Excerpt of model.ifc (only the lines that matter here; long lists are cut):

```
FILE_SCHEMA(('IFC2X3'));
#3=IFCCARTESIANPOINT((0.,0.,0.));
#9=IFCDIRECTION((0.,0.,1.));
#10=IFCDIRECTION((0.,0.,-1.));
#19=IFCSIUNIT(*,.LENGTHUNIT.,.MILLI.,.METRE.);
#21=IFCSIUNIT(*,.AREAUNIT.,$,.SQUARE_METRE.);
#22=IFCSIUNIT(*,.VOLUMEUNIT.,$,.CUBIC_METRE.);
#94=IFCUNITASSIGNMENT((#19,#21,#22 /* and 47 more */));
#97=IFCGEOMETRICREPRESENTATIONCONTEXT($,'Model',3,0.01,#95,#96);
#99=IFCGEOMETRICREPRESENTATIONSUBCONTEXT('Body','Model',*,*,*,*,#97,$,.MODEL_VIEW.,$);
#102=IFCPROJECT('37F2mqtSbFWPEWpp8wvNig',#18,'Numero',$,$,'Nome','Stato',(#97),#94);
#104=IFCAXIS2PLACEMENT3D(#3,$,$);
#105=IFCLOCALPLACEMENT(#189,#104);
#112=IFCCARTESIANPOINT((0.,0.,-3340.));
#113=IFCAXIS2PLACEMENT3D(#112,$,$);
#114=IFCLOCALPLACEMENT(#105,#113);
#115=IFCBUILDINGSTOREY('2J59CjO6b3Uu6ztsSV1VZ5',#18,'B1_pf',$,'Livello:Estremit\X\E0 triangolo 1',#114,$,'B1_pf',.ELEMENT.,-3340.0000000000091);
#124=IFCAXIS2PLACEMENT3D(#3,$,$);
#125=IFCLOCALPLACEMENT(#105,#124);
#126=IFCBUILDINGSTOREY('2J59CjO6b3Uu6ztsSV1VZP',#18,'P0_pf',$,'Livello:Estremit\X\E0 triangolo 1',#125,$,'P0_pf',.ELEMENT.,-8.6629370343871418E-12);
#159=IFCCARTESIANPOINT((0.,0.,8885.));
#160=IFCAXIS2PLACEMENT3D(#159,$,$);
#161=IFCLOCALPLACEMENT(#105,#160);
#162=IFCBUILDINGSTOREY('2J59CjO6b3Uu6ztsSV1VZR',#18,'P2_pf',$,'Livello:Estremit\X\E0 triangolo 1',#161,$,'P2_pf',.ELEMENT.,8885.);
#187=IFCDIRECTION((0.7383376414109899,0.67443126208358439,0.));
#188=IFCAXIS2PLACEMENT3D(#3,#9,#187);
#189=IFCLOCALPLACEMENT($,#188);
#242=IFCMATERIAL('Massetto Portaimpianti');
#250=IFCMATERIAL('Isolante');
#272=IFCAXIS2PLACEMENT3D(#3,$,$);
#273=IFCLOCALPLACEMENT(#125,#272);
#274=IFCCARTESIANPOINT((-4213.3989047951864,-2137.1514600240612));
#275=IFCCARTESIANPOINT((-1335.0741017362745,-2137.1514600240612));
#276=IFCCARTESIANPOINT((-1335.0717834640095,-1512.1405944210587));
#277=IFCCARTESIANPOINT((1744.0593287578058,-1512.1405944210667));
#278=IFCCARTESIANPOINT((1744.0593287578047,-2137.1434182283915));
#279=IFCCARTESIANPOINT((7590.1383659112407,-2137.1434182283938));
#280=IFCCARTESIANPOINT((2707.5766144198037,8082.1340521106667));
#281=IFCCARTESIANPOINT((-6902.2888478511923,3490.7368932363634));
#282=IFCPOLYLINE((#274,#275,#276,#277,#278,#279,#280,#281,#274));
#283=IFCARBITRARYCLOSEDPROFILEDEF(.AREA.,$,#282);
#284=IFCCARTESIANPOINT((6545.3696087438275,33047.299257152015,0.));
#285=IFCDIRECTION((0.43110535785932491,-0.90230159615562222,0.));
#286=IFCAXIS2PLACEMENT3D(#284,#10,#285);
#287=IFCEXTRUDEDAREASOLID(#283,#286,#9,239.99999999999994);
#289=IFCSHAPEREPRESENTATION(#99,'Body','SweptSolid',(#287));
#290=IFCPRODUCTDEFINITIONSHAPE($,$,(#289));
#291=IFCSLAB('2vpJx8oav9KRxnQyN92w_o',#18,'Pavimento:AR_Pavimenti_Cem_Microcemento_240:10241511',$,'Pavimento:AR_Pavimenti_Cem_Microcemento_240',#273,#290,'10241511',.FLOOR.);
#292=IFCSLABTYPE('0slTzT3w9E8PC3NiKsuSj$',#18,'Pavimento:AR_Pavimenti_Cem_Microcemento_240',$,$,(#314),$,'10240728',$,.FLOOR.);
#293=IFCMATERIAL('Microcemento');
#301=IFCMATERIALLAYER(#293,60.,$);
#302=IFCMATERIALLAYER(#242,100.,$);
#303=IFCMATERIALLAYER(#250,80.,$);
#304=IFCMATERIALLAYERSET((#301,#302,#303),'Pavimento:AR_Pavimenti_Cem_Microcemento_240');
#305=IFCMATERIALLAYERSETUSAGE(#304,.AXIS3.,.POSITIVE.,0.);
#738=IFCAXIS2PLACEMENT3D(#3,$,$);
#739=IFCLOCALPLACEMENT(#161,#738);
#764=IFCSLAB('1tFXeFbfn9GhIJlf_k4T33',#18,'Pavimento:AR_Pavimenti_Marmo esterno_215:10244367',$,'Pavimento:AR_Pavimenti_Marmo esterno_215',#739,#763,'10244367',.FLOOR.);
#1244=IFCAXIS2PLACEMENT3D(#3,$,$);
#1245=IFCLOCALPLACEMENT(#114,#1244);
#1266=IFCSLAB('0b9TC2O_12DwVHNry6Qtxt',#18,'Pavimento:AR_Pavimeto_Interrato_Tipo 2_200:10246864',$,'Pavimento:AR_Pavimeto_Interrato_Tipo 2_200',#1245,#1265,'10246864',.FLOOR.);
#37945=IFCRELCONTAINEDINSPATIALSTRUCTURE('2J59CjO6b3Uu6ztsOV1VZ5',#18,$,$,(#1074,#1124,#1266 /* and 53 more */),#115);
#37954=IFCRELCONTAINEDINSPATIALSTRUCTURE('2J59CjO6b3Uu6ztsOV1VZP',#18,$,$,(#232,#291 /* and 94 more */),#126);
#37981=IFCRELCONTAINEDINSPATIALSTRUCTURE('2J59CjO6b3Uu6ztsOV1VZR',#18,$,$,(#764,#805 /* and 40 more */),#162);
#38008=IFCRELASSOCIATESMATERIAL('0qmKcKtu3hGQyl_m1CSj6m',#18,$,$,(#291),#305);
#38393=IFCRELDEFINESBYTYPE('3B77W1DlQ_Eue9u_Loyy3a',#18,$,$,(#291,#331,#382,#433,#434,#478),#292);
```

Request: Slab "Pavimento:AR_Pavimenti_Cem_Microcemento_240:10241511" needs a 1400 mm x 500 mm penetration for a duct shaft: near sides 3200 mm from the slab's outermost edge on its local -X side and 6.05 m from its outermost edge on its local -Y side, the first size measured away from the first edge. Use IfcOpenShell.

```python
import numpy as np
import ifcopenshell
import ifcopenshell.api.feature
import ifcopenshell.api.geometry
import ifcopenshell.api.root
import ifcopenshell.geom
import ifcopenshell.util.placement
import ifcopenshell.util.representation
import ifcopenshell.util.shape
import ifcopenshell.util.unit

model = ifcopenshell.open("model.ifc")
unit_scale = ifcopenshell.util.unit.calculate_unit_scale(model)
settings = ifcopenshell.geom.settings()


def volume(element):
    """Net volume in cubic metres, openings subtracted."""
    shape = ifcopenshell.geom.create_shape(settings, element)
    return ifcopenshell.util.shape.get_volume(shape.geometry)


slab = model.by_guid("2vpJx8oav9KRxnQyN92w_o")
before = volume(slab)

# Extent in the slab's own axes, in metres. The edges named are its -X and -Y sides.
slab_shape = ifcopenshell.geom.create_shape(settings, slab)
vertices = ifcopenshell.util.shape.get_vertices(slab_shape.geometry)
x_min, y_min, bottom = vertices.min(axis=0)
top = vertices[:, 2].max()

opening = ifcopenshell.api.root.create_entity(model, ifc_class="IfcOpeningElement", name="Duct shaft opening")
context = ifcopenshell.util.representation.get_context(model, "Model", "Body", "MODEL_VIEW")
width, depth = 1.4, 0.5
outline = [(0.0, 0.0), (width, 0.0), (width, depth), (0.0, depth), (0.0, 0.0)]
# Overshoot both faces by 50 mm so the cut is clean.
shape = ifcopenshell.api.geometry.add_slab_representation(
    model, context=context, depth=top - bottom + 0.1, polyline=outline
)
ifcopenshell.api.geometry.assign_representation(model, product=opening, representation=shape)

matrix = ifcopenshell.util.placement.get_local_placement(slab.ObjectPlacement)
matrix[:, 3] = matrix @ np.append(np.array([x_min + 3.2, y_min + 6.05, bottom - 0.05]) / unit_scale, 1.0)
ifcopenshell.api.geometry.edit_object_placement(model, product=opening, matrix=matrix, is_si=False)
ifcopenshell.api.feature.add_feature(model, feature=opening, element=slab)

after = volume(slab)

print(f"slab volume {before:.3f} -> {after:.3f} m3")

model.write("model_rev.ifc")
```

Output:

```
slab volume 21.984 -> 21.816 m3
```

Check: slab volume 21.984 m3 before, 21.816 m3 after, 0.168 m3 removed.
